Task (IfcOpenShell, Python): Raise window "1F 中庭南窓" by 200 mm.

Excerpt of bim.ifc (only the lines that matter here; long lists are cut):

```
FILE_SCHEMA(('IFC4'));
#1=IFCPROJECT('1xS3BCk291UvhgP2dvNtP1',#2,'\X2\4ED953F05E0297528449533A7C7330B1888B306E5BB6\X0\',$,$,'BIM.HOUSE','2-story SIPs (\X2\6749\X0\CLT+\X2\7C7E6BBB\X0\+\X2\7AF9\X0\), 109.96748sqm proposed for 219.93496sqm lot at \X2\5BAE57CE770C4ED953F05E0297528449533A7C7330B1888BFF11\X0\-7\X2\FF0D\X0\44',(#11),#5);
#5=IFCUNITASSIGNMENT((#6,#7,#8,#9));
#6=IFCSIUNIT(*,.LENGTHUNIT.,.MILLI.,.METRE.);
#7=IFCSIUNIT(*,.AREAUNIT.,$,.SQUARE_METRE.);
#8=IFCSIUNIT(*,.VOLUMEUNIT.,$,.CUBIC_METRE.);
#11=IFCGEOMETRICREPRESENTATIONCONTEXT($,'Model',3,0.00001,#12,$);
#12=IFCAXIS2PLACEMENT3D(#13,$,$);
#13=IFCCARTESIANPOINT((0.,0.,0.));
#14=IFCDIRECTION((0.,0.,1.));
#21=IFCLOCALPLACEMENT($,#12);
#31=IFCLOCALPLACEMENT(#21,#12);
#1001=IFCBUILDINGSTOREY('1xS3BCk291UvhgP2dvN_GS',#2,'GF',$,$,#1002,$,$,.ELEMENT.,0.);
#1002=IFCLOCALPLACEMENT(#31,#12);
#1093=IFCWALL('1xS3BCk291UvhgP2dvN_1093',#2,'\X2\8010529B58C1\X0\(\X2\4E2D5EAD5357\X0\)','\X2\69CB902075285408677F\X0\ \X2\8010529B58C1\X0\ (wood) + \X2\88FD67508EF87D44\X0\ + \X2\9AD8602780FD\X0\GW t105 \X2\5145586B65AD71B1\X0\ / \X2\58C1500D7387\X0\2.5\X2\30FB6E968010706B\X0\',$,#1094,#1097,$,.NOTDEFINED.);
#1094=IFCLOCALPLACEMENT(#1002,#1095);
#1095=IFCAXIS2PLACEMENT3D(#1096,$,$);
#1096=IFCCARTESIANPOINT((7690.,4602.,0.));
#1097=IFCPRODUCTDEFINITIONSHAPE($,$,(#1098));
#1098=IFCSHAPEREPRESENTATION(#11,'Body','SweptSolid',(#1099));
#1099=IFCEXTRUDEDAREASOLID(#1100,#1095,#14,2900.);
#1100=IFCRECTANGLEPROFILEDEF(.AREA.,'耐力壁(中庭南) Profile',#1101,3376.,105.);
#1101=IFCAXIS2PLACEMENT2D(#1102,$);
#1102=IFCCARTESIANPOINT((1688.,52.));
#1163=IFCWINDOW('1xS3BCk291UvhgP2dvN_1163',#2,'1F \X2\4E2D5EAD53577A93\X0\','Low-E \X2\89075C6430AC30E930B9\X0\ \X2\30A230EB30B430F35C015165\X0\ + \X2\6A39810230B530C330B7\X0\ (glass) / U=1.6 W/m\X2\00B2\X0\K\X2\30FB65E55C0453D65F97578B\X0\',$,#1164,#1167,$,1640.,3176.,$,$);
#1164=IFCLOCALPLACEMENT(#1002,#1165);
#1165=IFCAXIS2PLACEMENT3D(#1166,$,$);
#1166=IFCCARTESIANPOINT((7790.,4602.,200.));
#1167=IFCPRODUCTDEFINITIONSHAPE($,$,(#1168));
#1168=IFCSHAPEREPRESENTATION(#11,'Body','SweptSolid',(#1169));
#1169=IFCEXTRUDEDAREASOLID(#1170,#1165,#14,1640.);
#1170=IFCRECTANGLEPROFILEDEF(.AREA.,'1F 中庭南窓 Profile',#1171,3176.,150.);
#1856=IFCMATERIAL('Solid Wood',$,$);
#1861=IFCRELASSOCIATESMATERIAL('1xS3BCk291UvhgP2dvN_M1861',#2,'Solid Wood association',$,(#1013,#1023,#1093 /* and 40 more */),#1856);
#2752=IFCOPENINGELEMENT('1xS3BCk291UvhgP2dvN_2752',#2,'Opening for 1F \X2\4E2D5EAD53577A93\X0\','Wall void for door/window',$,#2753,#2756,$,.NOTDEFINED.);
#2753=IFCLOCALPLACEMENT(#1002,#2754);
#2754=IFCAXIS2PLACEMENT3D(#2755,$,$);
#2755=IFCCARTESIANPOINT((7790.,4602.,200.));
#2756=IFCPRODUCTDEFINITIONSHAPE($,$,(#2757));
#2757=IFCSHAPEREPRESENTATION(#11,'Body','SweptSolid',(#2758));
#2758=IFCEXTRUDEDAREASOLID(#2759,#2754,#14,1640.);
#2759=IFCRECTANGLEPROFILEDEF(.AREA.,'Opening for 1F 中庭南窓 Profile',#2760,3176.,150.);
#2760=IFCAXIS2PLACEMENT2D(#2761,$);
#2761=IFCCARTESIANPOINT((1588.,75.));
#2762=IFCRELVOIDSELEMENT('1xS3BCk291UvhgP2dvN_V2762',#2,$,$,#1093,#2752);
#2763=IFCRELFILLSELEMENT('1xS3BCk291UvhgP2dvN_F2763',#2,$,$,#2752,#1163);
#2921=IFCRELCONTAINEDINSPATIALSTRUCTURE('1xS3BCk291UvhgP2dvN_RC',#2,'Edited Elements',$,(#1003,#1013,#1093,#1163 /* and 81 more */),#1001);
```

```python
import numpy as np
import ifcopenshell
import ifcopenshell.api.geometry
import ifcopenshell.util.placement
import ifcopenshell.util.unit

model = ifcopenshell.open("bim.ifc")
unit_scale = ifcopenshell.util.unit.calculate_unit_scale(model)

window = model.by_guid("1xS3BCk291UvhgP2dvN_1163")
opening = window.FillsVoids[0].RelatingOpeningElement
dz = 0.2 / unit_scale

shift = np.array([0.0, 0.0, dz])
# The window is not placed relative to its opening, so move both.
for product in (opening, window):
    matrix = ifcopenshell.util.placement.get_local_placement(product.ObjectPlacement)
    matrix[:3, 3] += shift
    ifcopenshell.api.geometry.edit_object_placement(model, product=product, matrix=matrix, is_si=False)

print(f"moved by {dz * unit_scale:+.3f} m")

model.write("bim-out.ifc")
```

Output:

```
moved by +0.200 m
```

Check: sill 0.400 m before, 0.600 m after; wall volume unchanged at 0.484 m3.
